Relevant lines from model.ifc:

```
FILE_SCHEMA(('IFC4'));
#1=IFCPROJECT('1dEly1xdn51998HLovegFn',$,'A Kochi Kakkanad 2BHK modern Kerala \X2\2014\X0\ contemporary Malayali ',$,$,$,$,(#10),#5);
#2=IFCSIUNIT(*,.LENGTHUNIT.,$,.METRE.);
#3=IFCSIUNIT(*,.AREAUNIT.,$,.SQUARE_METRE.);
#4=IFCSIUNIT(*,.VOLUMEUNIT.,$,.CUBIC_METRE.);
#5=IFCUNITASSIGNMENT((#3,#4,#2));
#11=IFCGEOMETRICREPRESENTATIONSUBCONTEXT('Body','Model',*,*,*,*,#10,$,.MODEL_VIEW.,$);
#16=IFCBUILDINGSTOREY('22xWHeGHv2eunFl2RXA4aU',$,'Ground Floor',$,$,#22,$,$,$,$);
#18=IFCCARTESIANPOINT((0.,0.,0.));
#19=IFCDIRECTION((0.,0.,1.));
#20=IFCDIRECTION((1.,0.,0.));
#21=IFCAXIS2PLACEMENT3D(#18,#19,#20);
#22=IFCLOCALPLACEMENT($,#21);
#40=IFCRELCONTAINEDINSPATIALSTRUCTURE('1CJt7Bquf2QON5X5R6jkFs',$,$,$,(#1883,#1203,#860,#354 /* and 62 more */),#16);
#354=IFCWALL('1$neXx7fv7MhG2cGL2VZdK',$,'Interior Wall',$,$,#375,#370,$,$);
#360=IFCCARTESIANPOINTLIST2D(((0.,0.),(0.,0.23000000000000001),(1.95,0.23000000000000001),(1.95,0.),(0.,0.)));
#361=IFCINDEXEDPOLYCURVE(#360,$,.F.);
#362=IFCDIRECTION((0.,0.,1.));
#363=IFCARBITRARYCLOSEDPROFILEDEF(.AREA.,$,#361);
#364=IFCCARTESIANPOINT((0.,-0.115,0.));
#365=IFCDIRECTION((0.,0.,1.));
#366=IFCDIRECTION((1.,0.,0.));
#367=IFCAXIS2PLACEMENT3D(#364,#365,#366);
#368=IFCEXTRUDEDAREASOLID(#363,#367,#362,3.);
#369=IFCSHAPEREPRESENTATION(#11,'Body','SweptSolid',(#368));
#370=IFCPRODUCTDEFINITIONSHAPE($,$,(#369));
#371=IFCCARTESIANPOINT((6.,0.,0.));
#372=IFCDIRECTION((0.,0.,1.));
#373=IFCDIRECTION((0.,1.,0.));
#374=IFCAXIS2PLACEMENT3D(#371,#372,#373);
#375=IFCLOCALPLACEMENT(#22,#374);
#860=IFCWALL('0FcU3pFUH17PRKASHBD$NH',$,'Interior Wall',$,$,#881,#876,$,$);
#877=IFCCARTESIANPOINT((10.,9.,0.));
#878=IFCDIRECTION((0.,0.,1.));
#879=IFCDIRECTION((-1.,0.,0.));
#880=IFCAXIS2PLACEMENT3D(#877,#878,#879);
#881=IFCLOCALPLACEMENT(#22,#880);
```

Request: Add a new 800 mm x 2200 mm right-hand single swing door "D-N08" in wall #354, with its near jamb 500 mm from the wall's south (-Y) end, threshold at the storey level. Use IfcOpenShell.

```python
import numpy as np
import ifcopenshell
import ifcopenshell.api.feature
import ifcopenshell.api.geometry
import ifcopenshell.api.root
import ifcopenshell.api.spatial
import ifcopenshell.geom
import ifcopenshell.util.element
import ifcopenshell.util.placement
import ifcopenshell.util.representation
import ifcopenshell.util.shape
import ifcopenshell.util.unit

model = ifcopenshell.open("model.ifc")
unit_scale = ifcopenshell.util.unit.calculate_unit_scale(model)
settings = ifcopenshell.geom.settings()


def volume(element):
    """Net volume in cubic metres, openings subtracted."""
    shape = ifcopenshell.geom.create_shape(settings, element)
    return ifcopenshell.util.shape.get_volume(shape.geometry)


wall = model.by_guid("1$neXx7fv7MhG2cGL2VZdK")
storey = ifcopenshell.util.element.get_container(wall, ifc_class="IfcBuildingStorey")
context = ifcopenshell.util.representation.get_context(model, "Model", "Body", "MODEL_VIEW")
before = volume(wall)

width, height, from_end, sill = 0.8, 2.2, 0.5, 0.0  # metres

# The wall runs along its own X axis, and the end named is its -X end.
wall_shape = ifcopenshell.geom.create_shape(settings, wall)
x, y, z = ifcopenshell.util.shape.get_vertices(wall_shape.geometry).T
start = x.min() + from_end
face, thickness = float(y.min()), float(y.max() - y.min())
wall_matrix = ifcopenshell.util.placement.get_local_placement(wall.ObjectPlacement)
level = ifcopenshell.util.placement.get_local_placement(storey.ObjectPlacement)[2, 3]


def in_wall(x, y):
    """Placement at x, y metres in the wall's axes, at sill height."""
    matrix = wall_matrix.copy()
    matrix[:, 3] = wall_matrix @ np.array([x / unit_scale, y / unit_scale, 0.0, 1.0])
    matrix[2, 3] = level + sill / unit_scale
    return matrix


# Opening: a box that overshoots both wall faces by 50 mm.
opening = ifcopenshell.api.root.create_entity(model, ifc_class="IfcOpeningElement", predefined_type="OPENING")
box = ifcopenshell.api.geometry.add_wall_representation(
    model, context=context, length=width, height=height, thickness=thickness + 0.1
)
ifcopenshell.api.geometry.assign_representation(model, product=opening, representation=box)
ifcopenshell.api.geometry.edit_object_placement(model, product=opening, matrix=in_wall(start, face - 0.05), is_si=False)
ifcopenshell.api.feature.add_feature(model, feature=opening, element=wall)

door = ifcopenshell.api.root.create_entity(model, ifc_class="IfcDoor", name="D-N08", predefined_type="DOOR")
door.OverallWidth, door.OverallHeight = width / unit_scale, height / unit_scale
door.OperationType = "SINGLE_SWING_RIGHT"
body = ifcopenshell.api.geometry.add_door_representation(
    model,
    context=context,
    overall_width=door.OverallWidth,
    overall_height=door.OverallHeight,
    operation_type="SINGLE_SWING_RIGHT",
    lining_properties={"LiningDepth": thickness / unit_scale, "ThresholdDepth": thickness / unit_scale},
)
ifcopenshell.api.geometry.assign_representation(model, product=door, representation=body)
ifcopenshell.api.spatial.assign_container(model, products=[door], relating_structure=storey)
ifcopenshell.api.feature.add_filling(model, opening=opening, element=door)

# The lining spans the wall, so the door starts at the wall face.
ifcopenshell.api.geometry.edit_object_placement(model, product=door, matrix=in_wall(start, face), is_si=False)

after = volume(wall)

print(f"wall volume {before:.3f} -> {after:.3f} m3")

model.write("model_updated.ifc")
```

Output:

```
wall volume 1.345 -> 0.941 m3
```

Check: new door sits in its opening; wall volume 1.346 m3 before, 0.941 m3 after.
